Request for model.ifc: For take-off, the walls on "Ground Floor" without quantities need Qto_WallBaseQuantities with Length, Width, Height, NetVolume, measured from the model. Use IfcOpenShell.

First a look at what the model holds.

```python
import ifcopenshell
import ifcopenshell.util.element
import ifcopenshell.util.unit

model = ifcopenshell.open("model.ifc")
print(model.schema)
for unit_type in ("LENGTHUNIT", "AREAUNIT", "VOLUMEUNIT"):
    print(unit_type, ifcopenshell.util.unit.calculate_unit_scale(model, unit_type))
storey = next(s for s in model.by_type("IfcBuildingStorey") if s.Name == "Ground Floor")
walls = [e for e in ifcopenshell.util.element.get_decomposition(storey) if e.is_a("IfcWall")]
for e in sorted(walls, key=lambda e: e.id()):
    print(e.id(), e.is_a(), e.Name, list(ifcopenshell.util.element.get_psets(e, qtos_only=True)), sep=" | ")
```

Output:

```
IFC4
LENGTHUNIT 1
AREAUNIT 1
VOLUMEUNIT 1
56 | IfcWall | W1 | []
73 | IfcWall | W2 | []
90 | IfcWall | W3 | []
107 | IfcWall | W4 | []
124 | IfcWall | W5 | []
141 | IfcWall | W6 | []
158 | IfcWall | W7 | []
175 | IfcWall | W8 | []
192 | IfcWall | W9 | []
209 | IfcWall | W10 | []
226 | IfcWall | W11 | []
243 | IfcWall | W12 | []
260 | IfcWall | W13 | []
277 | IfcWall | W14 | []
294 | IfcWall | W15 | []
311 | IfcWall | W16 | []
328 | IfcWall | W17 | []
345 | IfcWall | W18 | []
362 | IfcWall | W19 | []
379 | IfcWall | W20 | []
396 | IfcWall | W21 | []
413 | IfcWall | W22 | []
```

```python
import ifcopenshell
import ifcopenshell.api.pset
import ifcopenshell.geom
import ifcopenshell.util.element
import ifcopenshell.util.shape
import ifcopenshell.util.unit

model = ifcopenshell.open("model.ifc")
unit_scale = ifcopenshell.util.unit.calculate_unit_scale(model)
volume_scale = ifcopenshell.util.unit.calculate_unit_scale(model, "VOLUMEUNIT")
settings = ifcopenshell.geom.settings()

storey = next(s for s in model.by_type("IfcBuildingStorey") if s.Name == "Ground Floor")
walls = [e for e in ifcopenshell.util.element.get_decomposition(storey) if e.is_a("IfcWall")]

for e in sorted(walls, key=lambda e: e.id()):
    if ifcopenshell.util.element.get_psets(e, qtos_only=True, should_inherit=False):
        continue
    # Geometry comes back in metres, in the element's own axes.
    shape = ifcopenshell.geom.create_shape(settings, e)
    values = {
        "Length": ifcopenshell.util.shape.get_x(shape.geometry) / unit_scale,
        "Width": ifcopenshell.util.shape.get_y(shape.geometry) / unit_scale,
        "Height": ifcopenshell.util.shape.get_z(shape.geometry) / unit_scale,
        "NetVolume": ifcopenshell.util.shape.get_volume(shape.geometry) / volume_scale,
    }
    qto = ifcopenshell.api.pset.add_qto(model, product=e, name="Qto_WallBaseQuantities")
    ifcopenshell.api.pset.edit_qto(model, qto=qto, properties=values)
    print(e.id(), {k: round(v, 3) for k, v in values.items()})

model.write("model_v2.ifc")
```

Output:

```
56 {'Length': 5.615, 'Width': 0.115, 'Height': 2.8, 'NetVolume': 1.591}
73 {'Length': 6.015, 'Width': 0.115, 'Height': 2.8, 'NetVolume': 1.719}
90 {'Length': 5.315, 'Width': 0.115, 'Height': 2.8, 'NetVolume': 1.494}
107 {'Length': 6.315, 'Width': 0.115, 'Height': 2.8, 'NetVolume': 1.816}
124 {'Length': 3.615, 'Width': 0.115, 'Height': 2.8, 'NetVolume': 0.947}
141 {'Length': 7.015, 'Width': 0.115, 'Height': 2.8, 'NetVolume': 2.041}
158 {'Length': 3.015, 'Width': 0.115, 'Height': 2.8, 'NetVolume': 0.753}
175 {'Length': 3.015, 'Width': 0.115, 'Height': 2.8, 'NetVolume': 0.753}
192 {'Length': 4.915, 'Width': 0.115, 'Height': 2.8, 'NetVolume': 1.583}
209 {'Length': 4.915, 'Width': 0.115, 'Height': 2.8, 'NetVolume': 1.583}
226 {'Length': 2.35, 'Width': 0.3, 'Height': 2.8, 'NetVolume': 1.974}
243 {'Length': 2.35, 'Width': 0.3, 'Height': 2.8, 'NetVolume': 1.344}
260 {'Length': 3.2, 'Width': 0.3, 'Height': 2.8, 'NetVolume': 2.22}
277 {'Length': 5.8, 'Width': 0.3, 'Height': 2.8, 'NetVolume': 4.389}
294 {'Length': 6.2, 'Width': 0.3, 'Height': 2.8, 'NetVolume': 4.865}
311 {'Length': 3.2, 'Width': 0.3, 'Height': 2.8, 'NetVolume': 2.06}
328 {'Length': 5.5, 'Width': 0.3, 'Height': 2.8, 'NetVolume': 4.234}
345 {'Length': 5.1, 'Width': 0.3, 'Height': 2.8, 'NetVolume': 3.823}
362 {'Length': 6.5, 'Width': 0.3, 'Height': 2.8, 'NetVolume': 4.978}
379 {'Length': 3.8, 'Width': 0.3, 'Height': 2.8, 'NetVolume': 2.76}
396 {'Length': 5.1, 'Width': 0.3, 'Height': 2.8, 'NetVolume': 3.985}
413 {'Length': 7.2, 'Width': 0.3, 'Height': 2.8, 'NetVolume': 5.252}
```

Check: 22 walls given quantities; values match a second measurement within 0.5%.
